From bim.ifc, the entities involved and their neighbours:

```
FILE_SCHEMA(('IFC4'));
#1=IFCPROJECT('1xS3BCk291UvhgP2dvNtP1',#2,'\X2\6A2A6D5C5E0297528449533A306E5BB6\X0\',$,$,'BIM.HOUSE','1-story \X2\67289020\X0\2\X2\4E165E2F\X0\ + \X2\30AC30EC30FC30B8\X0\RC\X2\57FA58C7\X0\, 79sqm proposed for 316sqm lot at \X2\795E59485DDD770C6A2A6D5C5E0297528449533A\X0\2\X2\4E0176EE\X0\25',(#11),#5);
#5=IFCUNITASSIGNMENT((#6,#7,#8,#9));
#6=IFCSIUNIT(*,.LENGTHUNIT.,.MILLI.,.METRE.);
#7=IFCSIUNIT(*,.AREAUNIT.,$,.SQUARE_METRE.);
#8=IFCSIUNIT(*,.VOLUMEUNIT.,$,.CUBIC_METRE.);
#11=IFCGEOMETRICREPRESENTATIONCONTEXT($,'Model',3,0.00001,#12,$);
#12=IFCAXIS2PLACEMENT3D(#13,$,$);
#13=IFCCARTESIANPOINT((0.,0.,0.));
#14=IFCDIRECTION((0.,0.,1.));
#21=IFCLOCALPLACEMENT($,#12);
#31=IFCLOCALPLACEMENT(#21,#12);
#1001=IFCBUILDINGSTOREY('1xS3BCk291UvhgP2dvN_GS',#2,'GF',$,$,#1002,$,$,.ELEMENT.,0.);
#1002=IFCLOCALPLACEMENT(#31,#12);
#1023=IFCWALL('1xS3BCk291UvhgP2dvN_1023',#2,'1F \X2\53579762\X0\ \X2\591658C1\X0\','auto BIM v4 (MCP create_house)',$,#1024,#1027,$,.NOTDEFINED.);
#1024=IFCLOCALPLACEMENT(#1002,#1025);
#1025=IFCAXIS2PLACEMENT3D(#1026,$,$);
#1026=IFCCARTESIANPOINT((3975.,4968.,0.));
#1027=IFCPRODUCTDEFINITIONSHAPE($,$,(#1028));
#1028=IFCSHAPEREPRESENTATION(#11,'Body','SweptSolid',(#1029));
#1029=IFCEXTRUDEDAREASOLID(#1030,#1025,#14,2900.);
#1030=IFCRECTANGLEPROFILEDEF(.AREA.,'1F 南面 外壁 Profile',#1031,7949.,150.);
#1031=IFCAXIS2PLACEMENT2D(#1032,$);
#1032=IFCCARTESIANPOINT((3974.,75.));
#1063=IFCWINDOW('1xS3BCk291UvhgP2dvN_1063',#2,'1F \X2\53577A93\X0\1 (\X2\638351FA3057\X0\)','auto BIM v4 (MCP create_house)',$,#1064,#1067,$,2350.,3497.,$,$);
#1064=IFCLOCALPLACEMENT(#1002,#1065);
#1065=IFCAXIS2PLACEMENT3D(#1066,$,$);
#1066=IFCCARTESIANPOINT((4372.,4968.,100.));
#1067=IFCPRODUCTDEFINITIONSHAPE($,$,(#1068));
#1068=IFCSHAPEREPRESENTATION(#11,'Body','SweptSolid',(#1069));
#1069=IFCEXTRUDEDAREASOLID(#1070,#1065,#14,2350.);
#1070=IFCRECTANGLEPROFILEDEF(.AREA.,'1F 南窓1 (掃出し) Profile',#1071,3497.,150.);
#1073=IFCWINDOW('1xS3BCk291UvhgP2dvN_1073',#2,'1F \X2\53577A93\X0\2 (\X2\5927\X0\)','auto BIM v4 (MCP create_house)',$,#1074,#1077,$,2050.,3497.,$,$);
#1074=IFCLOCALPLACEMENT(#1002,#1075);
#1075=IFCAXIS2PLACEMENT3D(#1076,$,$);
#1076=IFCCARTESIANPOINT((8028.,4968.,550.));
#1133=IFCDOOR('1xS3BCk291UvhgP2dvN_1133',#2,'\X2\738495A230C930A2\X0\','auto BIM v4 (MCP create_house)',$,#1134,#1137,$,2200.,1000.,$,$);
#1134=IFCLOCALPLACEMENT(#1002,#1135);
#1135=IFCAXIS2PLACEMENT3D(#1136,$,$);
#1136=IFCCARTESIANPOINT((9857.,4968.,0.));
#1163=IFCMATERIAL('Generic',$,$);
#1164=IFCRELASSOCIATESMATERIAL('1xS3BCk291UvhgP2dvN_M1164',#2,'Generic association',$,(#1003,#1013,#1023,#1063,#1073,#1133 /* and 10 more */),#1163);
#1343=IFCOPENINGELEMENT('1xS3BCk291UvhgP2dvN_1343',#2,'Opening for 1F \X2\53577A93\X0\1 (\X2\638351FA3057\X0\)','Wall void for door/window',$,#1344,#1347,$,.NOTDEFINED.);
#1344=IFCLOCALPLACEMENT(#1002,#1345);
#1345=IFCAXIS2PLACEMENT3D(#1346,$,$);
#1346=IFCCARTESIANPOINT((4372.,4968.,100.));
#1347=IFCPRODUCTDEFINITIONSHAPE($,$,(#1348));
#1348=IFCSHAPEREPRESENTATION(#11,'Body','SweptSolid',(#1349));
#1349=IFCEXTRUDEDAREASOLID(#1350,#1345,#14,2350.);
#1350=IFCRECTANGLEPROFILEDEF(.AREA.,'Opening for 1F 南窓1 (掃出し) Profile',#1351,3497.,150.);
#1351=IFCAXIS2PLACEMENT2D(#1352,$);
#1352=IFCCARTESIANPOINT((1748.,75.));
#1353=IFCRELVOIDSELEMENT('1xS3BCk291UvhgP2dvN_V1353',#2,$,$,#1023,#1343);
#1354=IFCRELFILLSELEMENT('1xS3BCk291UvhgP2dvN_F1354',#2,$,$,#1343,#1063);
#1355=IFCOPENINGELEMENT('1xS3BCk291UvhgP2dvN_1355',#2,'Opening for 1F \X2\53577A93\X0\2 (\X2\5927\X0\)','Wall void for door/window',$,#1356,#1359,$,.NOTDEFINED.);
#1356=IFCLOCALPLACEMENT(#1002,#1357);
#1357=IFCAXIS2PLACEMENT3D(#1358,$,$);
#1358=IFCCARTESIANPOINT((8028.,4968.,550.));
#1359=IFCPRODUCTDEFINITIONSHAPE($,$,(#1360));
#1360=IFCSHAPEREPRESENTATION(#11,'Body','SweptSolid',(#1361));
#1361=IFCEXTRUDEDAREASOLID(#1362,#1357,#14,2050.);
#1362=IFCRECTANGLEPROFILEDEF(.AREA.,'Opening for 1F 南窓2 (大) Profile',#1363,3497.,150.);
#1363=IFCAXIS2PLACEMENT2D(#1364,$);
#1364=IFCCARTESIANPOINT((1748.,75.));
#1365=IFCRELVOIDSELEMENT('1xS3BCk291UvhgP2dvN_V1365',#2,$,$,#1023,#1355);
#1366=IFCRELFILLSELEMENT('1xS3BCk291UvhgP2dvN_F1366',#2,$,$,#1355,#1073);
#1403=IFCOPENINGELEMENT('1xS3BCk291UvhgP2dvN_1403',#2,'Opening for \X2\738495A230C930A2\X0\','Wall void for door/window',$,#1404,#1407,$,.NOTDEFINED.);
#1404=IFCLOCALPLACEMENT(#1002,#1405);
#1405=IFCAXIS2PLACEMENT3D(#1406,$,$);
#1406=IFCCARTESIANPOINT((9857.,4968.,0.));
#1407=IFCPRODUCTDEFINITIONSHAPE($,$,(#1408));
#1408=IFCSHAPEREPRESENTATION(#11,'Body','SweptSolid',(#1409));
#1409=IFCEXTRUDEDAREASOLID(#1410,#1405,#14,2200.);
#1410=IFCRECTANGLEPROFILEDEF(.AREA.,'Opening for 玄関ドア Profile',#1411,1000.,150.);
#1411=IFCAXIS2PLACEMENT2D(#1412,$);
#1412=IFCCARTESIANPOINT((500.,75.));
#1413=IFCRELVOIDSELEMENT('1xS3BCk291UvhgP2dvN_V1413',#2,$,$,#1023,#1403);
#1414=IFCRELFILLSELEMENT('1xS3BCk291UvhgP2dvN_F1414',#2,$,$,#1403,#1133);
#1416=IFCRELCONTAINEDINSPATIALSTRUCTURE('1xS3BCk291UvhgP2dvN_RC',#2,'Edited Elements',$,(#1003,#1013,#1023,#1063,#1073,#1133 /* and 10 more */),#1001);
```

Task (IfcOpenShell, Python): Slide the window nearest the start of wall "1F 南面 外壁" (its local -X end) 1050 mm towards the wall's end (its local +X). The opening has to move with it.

```python
import ifcopenshell
import ifcopenshell.api.geometry
import ifcopenshell.util.placement
import ifcopenshell.util.unit

model = ifcopenshell.open("bim.ifc")
unit_scale = ifcopenshell.util.unit.calculate_unit_scale(model)

window = model.by_id(1063)
opening = window.FillsVoids[0].RelatingOpeningElement
wall = opening.VoidsElements[0].RelatingBuildingElement

wall_matrix = ifcopenshell.util.placement.get_local_placement(wall.ObjectPlacement)
shift = wall_matrix[:3, 0] * 1.05 / unit_scale
before = ifcopenshell.util.placement.get_local_placement(window.ObjectPlacement)[:3, 3].copy()

# The window is not placed relative to its opening, so move both.
for product in (opening, window):
    matrix = ifcopenshell.util.placement.get_local_placement(product.ObjectPlacement)
    matrix[:3, 3] += shift
    ifcopenshell.api.geometry.edit_object_placement(model, product=product, matrix=matrix, is_si=False)

after = ifcopenshell.util.placement.get_local_placement(window.ObjectPlacement)[:3, 3]
print("window moved by", (after - before).round(3) + 0.0)

model.write("bim_v2.ifc")
```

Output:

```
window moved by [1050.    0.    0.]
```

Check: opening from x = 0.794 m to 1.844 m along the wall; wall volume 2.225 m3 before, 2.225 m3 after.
